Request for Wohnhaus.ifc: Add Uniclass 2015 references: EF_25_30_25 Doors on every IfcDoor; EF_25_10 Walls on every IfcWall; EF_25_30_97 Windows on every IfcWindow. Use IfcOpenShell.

First a look at what the model holds.

```python
import ifcopenshell

model = ifcopenshell.open("Wohnhaus.ifc")
print(model.schema)
print("classifications:", [c.Name for c in model.by_type("IfcClassification")])
for ifc_class in ("IfcDoor", "IfcRoof", "IfcStair", "IfcWall", "IfcWindow"):
    print(ifc_class, len(model.by_type(ifc_class)))
```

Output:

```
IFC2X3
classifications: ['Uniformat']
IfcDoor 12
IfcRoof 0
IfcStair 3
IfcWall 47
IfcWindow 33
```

```python
import ifcopenshell
import ifcopenshell.api.classification

model = ifcopenshell.open("Wohnhaus.ifc")

# IFC2X3 requires Source and Edition and has no link from the project to the system.
system = model.create_entity("IfcClassification", Source="NBS", Edition="2015", Name="Uniclass 2015")

codes = {
    "IfcDoor": ("EF_25_30_25", "Doors"),
    "IfcWall": ("EF_25_10", "Walls"),
    "IfcWindow": ("EF_25_30_97", "Windows"),
}
for ifc_class, (code, name) in codes.items():
    products = model.by_type(ifc_class)
    ifcopenshell.api.classification.add_reference(
        model, products=products, classification=system, identification=code, name=name
    )
    print(code, len(products))

model.write("Wohnhaus_updated.ifc")
```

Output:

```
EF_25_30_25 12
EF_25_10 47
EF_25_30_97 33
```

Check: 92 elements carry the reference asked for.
